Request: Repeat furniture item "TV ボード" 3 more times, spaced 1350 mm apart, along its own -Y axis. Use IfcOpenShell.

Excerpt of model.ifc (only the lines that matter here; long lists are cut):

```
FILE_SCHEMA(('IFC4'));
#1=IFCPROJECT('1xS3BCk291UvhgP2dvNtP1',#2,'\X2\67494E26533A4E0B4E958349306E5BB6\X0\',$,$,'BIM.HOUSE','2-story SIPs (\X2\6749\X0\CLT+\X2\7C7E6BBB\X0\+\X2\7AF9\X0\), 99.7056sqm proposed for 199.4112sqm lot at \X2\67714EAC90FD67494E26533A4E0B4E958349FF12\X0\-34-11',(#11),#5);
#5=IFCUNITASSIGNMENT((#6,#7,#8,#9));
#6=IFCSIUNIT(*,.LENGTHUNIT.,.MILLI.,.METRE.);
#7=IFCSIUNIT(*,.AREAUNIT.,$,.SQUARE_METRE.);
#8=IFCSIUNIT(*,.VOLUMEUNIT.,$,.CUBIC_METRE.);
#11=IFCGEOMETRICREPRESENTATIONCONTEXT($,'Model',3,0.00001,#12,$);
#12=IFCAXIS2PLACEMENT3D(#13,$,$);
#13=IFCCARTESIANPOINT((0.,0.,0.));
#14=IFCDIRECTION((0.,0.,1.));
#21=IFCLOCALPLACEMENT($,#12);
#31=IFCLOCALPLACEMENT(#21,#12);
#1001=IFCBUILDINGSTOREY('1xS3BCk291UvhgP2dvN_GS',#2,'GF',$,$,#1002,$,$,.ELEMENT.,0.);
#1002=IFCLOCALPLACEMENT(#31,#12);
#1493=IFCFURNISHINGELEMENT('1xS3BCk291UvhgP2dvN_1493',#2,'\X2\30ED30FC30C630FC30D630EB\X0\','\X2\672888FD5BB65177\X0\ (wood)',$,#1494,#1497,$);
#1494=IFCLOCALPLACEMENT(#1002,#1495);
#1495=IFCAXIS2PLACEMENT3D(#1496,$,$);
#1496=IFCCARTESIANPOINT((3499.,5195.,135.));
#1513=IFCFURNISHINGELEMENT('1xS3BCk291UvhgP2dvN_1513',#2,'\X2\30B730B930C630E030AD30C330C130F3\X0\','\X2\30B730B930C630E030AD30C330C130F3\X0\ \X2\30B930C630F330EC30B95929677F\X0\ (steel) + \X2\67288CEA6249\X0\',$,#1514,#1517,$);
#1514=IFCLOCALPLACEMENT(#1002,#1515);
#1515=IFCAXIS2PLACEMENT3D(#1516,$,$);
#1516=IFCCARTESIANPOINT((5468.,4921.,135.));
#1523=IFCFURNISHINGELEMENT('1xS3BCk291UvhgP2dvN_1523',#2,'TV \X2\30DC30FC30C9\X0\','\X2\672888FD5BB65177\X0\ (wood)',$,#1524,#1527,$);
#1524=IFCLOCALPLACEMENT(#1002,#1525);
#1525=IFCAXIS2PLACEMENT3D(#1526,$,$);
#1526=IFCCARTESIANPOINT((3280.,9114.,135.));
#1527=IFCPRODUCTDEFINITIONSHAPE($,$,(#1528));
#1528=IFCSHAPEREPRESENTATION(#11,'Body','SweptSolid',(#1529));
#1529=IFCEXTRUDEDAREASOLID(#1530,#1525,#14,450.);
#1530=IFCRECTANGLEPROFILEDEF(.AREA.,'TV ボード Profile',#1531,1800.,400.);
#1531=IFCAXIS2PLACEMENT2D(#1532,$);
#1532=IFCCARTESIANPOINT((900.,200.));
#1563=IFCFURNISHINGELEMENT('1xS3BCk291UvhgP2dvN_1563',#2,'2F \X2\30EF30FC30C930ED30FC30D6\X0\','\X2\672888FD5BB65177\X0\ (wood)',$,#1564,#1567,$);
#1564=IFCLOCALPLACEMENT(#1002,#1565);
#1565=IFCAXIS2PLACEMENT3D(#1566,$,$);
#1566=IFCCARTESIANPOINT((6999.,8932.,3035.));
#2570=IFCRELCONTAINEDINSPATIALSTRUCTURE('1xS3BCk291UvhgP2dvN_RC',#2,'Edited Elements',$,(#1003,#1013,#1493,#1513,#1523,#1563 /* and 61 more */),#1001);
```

```python
import ifcopenshell
import ifcopenshell.api.geometry
import ifcopenshell.api.root
import ifcopenshell.util.element
import ifcopenshell.util.placement

model = ifcopenshell.open("model.ifc")


def reuse_history(source, copy):
    """copy_class also copies each property set's owner history, people and application; keep the originals."""
    for rel in copy.IsDefinedBy:
        if rel.is_a("IfcRelDefinesByProperties") and (history := rel.RelatingPropertyDefinition.OwnerHistory):
            rel.RelatingPropertyDefinition.OwnerHistory = source.OwnerHistory
            ifcopenshell.util.element.remove_deep2(model, history)


source = model.by_id(1523)
base = ifcopenshell.util.placement.get_local_placement(source.ObjectPlacement)
step = -base[:3, 1] * 1350.0

for i in range(1, 4):
    copy = ifcopenshell.api.root.copy_class(model, product=source)
    copy.Representation = ifcopenshell.util.element.copy_deep(
        model, source.Representation, exclude=["IfcGeometricRepresentationContext", "IfcRepresentationMap"]
    )
    reuse_history(source, copy)
    matrix = base.copy()
    matrix[:3, 3] += i * step
    print("added at", matrix[:3, 3].round(3) + 0.0)
    ifcopenshell.api.geometry.edit_object_placement(model, product=copy, matrix=matrix, is_si=False)

model.write("model_edited.ifc")
```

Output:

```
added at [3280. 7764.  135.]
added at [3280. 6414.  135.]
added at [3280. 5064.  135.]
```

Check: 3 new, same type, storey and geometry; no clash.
